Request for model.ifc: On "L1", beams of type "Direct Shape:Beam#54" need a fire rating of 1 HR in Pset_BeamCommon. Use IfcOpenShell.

First a look at what the model holds.

```python
import ifcopenshell
import ifcopenshell.util.element

model = ifcopenshell.open("model.ifc")
print(model.schema)
storey = next(s for s in model.by_type("IfcBuildingStorey") if s.Name == "L1")
beams = [e for e in ifcopenshell.util.element.get_decomposition(storey) if e.is_a("IfcBeam")]
seen = {}
for e in beams:
    element_type = ifcopenshell.util.element.get_type(e)
    key = (element_type.Name if element_type != e and element_type else None, ifcopenshell.util.element.get_pset(e, "Pset_BeamCommon", "FireRating"))
    seen[key] = seen.get(key, 0) + 1
for (name, value), count in sorted(seen.items(), key=str):
    print(count, "x", name, "|", value)
```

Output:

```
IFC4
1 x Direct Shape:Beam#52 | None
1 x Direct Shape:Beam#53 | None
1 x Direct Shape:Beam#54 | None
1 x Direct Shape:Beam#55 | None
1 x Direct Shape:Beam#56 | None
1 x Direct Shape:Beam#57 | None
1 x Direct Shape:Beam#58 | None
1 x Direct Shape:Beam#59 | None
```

```python
import ifcopenshell
import ifcopenshell.api.pset
import ifcopenshell.util.element

model = ifcopenshell.open("model.ifc")

storey = next(s for s in model.by_type("IfcBuildingStorey") if s.Name == "L1")
beams = [e for e in ifcopenshell.util.element.get_decomposition(storey) if e.is_a("IfcBeam")]

count = 0
for e in beams:
    element_type = ifcopenshell.util.element.get_type(e)
    if element_type in (None, e) or element_type.Name != "Direct Shape:Beam#54":
        continue
    # add_pset returns the element's existing set when there is one.
    pset = ifcopenshell.api.pset.add_pset(model, product=e, name="Pset_BeamCommon")
    ifcopenshell.api.pset.edit_pset(model, pset=pset, properties={"FireRating": "1 HR"})
    count += 1

print(count, "beams updated")

model.write("model_updated.ifc")
```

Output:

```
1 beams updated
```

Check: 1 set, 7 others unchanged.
